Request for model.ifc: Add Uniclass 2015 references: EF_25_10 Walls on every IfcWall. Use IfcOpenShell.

First a look at what the model holds.

```python
import ifcopenshell

model = ifcopenshell.open("model.ifc")
print(model.schema)
print("classifications:", [c.Name for c in model.by_type("IfcClassification")])
for ifc_class in ("IfcDoor", "IfcRoof", "IfcStair", "IfcWall", "IfcWindow"):
    print(ifc_class, len(model.by_type(ifc_class)))
```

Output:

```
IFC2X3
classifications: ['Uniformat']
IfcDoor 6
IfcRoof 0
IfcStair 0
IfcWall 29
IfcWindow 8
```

```python
import ifcopenshell
import ifcopenshell.api.classification

model = ifcopenshell.open("model.ifc")

# IFC2X3 requires Source and Edition and has no link from the project to the system.
system = model.create_entity("IfcClassification", Source="NBS", Edition="2015", Name="Uniclass 2015")

codes = {
    "IfcWall": ("EF_25_10", "Walls"),
}
for ifc_class, (code, name) in codes.items():
    products = model.by_type(ifc_class)
    ifcopenshell.api.classification.add_reference(
        model, products=products, classification=system, identification=code, name=name
    )
    print(code, len(products))

model.write("model_v2.ifc")
```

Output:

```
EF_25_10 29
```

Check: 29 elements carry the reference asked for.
